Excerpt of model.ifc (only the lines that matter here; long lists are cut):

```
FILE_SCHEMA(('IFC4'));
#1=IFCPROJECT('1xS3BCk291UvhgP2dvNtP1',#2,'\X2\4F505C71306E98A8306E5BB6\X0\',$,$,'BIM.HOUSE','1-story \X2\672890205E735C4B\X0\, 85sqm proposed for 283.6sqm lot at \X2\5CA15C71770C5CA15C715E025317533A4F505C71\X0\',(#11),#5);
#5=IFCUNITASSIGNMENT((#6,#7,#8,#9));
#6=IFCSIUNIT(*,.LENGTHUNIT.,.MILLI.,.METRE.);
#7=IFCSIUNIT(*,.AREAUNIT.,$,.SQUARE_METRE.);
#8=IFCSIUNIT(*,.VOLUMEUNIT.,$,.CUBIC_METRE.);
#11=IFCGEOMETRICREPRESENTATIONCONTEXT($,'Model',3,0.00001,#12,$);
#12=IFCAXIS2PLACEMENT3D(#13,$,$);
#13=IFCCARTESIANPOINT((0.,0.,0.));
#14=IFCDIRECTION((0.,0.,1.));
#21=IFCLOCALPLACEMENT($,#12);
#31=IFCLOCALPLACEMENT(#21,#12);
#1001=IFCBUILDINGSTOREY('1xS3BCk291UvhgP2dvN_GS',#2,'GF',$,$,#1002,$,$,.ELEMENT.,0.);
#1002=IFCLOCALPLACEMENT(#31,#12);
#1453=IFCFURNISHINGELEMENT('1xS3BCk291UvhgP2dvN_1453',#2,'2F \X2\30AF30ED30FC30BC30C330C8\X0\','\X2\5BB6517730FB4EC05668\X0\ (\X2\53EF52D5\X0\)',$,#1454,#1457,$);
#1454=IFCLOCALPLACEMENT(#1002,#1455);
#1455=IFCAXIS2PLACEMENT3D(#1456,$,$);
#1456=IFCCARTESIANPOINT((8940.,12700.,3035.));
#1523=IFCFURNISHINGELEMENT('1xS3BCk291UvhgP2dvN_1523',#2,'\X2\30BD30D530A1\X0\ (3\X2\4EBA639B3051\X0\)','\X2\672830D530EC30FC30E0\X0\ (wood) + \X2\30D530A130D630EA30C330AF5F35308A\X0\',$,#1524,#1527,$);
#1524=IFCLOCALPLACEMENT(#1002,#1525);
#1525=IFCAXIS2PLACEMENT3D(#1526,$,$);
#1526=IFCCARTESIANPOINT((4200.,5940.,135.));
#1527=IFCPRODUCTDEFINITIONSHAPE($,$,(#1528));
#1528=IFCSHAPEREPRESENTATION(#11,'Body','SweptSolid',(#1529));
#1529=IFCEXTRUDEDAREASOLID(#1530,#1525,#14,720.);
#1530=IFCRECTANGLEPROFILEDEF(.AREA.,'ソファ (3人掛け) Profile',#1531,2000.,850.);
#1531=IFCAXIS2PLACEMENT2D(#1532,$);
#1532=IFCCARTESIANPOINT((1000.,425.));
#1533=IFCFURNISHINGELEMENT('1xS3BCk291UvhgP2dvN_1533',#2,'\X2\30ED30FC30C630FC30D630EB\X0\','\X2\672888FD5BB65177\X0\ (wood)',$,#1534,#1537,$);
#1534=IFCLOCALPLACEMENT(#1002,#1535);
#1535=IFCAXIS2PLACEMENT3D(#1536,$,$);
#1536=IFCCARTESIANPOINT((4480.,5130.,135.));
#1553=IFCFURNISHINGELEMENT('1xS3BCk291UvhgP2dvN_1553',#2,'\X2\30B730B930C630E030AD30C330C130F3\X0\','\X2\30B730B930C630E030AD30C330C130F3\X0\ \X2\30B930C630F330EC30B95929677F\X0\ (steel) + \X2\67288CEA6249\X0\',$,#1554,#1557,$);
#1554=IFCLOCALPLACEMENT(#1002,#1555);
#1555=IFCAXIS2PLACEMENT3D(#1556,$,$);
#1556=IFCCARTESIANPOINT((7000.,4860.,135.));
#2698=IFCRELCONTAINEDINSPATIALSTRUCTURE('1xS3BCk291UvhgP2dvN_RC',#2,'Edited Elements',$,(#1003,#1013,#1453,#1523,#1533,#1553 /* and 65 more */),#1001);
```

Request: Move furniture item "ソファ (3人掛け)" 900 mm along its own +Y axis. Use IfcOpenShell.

```python
import ifcopenshell
import ifcopenshell.api.geometry
import ifcopenshell.util.placement

model = ifcopenshell.open("model.ifc")

item = model.by_guid("1xS3BCk291UvhgP2dvN_1523")
matrix = ifcopenshell.util.placement.get_local_placement(item.ObjectPlacement)
matrix[:3, 3] += matrix[:3, 1] * 900.0
ifcopenshell.api.geometry.edit_object_placement(model, product=item, matrix=matrix, is_si=False)

print(ifcopenshell.util.placement.get_local_placement(item.ObjectPlacement).round(3) + 0.0)

model.write("model-out.ifc")
```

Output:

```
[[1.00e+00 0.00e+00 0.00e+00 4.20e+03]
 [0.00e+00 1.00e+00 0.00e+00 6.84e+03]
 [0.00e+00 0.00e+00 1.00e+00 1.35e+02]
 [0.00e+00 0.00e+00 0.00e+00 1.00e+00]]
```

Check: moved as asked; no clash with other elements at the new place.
